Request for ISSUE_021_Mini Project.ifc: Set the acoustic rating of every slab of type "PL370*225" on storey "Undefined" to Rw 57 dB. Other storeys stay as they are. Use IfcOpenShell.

First a look at what the model holds.

```python
import ifcopenshell
import ifcopenshell.util.element

model = ifcopenshell.open("ISSUE_021_Mini Project.ifc")
print(model.schema)
storey = next(s for s in model.by_type("IfcBuildingStorey") if s.Name == "Undefined")
slabs = [e for e in ifcopenshell.util.element.get_decomposition(storey) if e.is_a("IfcSlab")]
seen = {}
for e in slabs:
    element_type = ifcopenshell.util.element.get_type(e)
    key = (element_type.Name if element_type != e and element_type else None, ifcopenshell.util.element.get_pset(e, "Pset_SlabCommon", "AcousticRating"))
    seen[key] = seen.get(key, 0) + 1
for (name, value), count in sorted(seen.items(), key=str):
    print(count, "x", name, "|", value)
```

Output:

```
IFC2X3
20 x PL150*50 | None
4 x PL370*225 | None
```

```python
import ifcopenshell
import ifcopenshell.api.pset
import ifcopenshell.util.element

model = ifcopenshell.open("ISSUE_021_Mini Project.ifc")

storey = next(s for s in model.by_type("IfcBuildingStorey") if s.Name == "Undefined")
slabs = [e for e in ifcopenshell.util.element.get_decomposition(storey) if e.is_a("IfcSlab")]

count = 0
for e in slabs:
    element_type = ifcopenshell.util.element.get_type(e)
    if element_type in (None, e) or element_type.Name != "PL370*225":
        continue
    found = ifcopenshell.util.element.get_pset(e, "Pset_SlabCommon", should_inherit=False)
    if found:
        pset = model.by_id(found["id"])
        if len(ifcopenshell.util.element.get_elements_by_pset(pset)) > 1:
            pset = ifcopenshell.api.pset.unshare_pset(model, products=[e], pset=pset)[0]
    else:
        pset = ifcopenshell.api.pset.add_pset(model, product=e, name="Pset_SlabCommon")
    ifcopenshell.api.pset.edit_pset(model, pset=pset, properties={"AcousticRating": "Rw 57 dB"})
    count += 1

print(count, "slabs updated")

model.write("ISSUE_021_Mini Project-out.ifc")
```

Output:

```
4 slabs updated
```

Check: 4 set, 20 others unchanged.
